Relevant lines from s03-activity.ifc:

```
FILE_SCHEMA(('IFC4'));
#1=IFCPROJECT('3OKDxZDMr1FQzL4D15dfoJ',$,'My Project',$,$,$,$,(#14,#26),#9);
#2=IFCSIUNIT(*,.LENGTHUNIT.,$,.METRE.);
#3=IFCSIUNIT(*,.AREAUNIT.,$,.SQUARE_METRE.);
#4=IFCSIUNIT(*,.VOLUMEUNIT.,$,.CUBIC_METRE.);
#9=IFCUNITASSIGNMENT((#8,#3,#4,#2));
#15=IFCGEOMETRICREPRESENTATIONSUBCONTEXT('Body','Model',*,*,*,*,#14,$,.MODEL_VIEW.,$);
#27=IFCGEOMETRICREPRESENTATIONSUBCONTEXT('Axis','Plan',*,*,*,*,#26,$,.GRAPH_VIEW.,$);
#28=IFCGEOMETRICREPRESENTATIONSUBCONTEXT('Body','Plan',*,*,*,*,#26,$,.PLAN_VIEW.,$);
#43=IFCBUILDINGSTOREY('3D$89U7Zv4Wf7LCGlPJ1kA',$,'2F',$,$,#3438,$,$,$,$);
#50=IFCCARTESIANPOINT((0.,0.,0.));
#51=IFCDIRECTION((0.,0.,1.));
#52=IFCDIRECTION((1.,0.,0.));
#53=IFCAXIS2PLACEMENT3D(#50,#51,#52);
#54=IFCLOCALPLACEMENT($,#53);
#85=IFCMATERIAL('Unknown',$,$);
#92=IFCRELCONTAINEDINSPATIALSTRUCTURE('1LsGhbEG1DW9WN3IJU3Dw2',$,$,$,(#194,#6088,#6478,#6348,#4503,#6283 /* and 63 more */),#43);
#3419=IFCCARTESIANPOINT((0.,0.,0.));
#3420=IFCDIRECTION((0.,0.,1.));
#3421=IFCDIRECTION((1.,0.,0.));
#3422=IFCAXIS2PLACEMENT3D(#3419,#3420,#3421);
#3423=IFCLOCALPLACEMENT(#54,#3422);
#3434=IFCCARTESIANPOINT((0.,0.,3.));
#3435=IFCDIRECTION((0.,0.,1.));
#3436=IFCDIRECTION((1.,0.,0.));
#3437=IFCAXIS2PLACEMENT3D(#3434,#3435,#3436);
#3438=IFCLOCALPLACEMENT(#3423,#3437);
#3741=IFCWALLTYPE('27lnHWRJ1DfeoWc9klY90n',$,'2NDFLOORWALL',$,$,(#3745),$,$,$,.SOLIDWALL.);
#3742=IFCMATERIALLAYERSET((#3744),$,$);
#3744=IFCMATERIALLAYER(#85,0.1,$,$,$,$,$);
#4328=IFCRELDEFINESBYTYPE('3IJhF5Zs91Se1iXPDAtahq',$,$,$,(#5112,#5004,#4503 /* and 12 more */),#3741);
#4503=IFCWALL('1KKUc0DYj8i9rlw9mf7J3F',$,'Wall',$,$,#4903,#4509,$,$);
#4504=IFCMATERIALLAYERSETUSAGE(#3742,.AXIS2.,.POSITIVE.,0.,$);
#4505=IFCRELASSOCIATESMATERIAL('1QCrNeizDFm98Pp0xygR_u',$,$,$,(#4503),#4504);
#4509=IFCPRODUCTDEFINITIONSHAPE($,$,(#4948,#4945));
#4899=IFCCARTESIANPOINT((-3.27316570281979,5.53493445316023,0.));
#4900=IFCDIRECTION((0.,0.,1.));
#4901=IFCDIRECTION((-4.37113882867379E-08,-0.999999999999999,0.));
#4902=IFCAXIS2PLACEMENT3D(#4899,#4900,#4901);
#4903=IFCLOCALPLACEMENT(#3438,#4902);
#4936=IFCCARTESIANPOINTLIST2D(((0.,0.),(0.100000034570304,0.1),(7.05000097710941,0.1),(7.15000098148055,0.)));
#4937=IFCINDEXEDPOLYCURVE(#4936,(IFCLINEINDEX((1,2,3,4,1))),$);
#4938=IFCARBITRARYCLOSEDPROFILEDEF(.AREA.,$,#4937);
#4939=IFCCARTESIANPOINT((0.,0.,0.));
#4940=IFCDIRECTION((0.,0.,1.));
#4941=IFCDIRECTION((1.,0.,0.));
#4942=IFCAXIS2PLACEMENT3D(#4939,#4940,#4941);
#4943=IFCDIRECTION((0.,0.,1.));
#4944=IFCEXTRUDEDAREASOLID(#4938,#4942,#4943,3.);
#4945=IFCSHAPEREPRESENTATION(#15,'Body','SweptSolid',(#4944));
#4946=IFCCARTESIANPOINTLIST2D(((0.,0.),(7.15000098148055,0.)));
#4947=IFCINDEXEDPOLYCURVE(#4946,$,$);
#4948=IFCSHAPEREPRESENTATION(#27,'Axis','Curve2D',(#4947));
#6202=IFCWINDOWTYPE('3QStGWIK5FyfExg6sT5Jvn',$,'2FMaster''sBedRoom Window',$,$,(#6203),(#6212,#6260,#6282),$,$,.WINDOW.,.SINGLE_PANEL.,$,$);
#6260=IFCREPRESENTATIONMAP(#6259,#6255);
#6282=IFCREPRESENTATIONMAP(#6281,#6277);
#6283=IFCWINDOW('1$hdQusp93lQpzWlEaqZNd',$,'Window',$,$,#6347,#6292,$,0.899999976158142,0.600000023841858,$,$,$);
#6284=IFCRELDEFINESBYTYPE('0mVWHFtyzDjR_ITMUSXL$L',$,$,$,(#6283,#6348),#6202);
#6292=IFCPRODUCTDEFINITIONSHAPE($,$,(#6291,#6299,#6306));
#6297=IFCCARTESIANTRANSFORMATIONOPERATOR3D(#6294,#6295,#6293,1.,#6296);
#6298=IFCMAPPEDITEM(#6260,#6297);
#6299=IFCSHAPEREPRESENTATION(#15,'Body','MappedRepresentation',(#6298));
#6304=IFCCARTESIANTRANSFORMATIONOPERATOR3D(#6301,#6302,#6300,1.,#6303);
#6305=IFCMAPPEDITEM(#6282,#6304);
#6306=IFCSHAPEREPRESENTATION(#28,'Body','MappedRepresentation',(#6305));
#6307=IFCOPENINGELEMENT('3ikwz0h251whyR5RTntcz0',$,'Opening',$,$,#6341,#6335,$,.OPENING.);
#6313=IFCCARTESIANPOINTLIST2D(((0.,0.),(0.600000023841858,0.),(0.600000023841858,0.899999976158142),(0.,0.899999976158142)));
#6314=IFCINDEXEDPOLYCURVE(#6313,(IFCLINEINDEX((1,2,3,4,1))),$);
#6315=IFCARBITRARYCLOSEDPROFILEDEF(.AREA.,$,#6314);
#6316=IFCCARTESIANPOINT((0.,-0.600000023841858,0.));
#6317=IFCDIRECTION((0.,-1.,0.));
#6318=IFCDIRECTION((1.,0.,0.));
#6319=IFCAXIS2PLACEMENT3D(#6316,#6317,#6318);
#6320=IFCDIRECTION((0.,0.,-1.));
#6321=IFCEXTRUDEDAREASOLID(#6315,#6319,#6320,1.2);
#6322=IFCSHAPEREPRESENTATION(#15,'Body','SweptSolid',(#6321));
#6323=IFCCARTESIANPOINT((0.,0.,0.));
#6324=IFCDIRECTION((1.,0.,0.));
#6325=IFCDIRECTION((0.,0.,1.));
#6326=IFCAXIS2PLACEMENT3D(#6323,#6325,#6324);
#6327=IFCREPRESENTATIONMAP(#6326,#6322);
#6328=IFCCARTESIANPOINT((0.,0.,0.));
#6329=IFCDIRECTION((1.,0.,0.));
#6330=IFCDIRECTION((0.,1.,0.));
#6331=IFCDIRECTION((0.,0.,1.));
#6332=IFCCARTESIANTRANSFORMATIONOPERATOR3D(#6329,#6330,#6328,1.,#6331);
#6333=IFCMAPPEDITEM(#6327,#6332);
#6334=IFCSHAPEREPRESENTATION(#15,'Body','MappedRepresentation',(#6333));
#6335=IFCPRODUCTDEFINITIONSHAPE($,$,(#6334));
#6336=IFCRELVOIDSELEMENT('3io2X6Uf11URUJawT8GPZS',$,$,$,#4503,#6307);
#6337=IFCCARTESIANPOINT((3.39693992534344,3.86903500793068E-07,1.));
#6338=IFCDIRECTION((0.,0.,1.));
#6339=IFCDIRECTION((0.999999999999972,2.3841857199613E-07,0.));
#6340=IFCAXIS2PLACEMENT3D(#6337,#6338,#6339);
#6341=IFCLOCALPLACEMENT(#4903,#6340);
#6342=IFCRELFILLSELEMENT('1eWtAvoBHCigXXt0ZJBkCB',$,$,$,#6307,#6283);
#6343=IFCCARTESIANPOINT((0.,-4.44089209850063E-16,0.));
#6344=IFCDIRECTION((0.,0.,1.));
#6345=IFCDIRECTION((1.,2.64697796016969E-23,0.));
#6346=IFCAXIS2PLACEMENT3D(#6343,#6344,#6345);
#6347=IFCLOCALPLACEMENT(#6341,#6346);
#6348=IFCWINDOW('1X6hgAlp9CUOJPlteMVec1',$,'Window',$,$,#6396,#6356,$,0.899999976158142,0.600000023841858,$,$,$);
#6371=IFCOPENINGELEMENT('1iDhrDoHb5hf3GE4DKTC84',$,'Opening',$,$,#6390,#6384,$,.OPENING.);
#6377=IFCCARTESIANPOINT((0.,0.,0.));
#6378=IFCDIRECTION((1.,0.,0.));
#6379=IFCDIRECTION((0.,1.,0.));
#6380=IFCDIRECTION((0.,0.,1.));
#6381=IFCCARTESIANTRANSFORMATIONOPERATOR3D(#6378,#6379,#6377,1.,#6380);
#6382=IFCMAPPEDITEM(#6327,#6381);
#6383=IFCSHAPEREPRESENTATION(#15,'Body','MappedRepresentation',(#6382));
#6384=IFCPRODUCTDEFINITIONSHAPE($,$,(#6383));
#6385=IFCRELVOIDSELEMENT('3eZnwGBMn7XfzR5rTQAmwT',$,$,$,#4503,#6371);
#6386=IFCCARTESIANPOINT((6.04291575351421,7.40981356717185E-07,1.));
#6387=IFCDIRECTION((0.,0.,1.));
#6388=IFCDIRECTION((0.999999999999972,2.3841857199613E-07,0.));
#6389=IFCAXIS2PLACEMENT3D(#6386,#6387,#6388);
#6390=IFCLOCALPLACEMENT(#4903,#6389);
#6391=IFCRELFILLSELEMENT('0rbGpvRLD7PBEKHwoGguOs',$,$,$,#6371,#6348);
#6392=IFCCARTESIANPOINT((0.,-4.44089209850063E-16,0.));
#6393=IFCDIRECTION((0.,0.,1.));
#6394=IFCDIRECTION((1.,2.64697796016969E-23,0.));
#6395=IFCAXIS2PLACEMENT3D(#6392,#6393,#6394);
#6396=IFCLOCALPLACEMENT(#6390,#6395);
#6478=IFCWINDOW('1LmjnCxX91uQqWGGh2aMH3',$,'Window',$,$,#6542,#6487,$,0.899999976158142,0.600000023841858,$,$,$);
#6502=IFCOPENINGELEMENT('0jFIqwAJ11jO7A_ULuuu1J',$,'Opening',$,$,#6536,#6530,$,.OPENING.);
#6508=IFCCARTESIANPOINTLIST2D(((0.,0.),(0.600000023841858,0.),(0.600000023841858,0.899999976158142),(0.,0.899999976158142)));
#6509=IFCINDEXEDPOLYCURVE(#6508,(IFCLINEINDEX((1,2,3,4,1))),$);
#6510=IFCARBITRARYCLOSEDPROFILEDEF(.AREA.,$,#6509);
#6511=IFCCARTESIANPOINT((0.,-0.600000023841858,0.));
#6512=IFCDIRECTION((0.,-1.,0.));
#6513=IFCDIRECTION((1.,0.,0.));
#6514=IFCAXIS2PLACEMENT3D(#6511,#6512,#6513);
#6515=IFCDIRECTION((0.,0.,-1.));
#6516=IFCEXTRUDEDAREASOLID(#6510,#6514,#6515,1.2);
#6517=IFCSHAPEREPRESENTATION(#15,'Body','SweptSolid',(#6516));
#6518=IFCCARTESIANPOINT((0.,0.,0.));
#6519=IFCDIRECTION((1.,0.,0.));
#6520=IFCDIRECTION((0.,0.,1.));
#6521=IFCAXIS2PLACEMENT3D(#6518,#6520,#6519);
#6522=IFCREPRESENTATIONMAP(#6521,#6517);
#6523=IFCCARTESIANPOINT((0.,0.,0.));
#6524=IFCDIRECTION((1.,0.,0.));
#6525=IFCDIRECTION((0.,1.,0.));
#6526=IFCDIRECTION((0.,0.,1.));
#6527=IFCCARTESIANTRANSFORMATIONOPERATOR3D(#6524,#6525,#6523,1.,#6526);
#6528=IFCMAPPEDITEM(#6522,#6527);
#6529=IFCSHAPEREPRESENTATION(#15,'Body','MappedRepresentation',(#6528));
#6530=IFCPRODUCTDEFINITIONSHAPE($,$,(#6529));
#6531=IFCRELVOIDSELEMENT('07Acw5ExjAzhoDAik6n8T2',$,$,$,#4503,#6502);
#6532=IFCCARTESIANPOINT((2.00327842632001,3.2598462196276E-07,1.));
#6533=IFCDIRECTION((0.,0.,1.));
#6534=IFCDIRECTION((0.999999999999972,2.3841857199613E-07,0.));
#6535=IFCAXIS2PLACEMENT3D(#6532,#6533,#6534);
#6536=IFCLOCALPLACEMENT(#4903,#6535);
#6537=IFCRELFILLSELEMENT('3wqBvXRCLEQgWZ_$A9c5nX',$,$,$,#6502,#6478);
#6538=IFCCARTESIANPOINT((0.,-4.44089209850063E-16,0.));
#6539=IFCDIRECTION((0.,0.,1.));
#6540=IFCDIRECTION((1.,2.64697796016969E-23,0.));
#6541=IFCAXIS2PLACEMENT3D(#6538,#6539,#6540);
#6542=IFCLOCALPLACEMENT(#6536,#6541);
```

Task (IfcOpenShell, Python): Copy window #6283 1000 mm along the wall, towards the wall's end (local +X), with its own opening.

```python
import ifcopenshell
import ifcopenshell.api.feature
import ifcopenshell.api.geometry
import ifcopenshell.api.root
import ifcopenshell.geom
import ifcopenshell.util.element
import ifcopenshell.util.placement
import ifcopenshell.util.shape
import ifcopenshell.util.unit

model = ifcopenshell.open("s03-activity.ifc")
unit_scale = ifcopenshell.util.unit.calculate_unit_scale(model)
settings = ifcopenshell.geom.settings()


def volume(element):
    """Net volume in cubic metres, openings subtracted."""
    shape = ifcopenshell.geom.create_shape(settings, element)
    return ifcopenshell.util.shape.get_volume(shape.geometry)


window = model.by_id(6283)
opening = window.FillsVoids[0].RelatingOpeningElement
wall = opening.VoidsElements[0].RelatingBuildingElement
before = volume(wall)
shift = ifcopenshell.util.placement.get_local_placement(wall.ObjectPlacement)[:3, 0] * 1 / unit_scale

# copy_class copies the void relationship, type, container and properties, but no geometry.
new_opening = ifcopenshell.api.root.copy_class(model, product=opening)
new_opening.Representation = ifcopenshell.util.element.copy_deep(
    model, opening.Representation, exclude=["IfcGeometricRepresentationContext", "IfcRepresentationMap"]
)
new_window = ifcopenshell.api.root.copy_class(model, product=window)
new_window.Representation = ifcopenshell.util.element.copy_deep(
    model, window.Representation, exclude=["IfcGeometricRepresentationContext", "IfcRepresentationMap"]
)
ifcopenshell.api.feature.add_filling(model, opening=new_opening, element=new_window)

for old, new in ((opening, new_opening), (window, new_window)):
    matrix = ifcopenshell.util.placement.get_local_placement(old.ObjectPlacement)
    matrix[:3, 3] += shift
    ifcopenshell.api.geometry.edit_object_placement(model, product=new, matrix=matrix, is_si=False)

after = volume(wall)

print(f"wall volume {before:.3f} -> {after:.3f} m3")

model.write("s03-activity_edited.ifc")
```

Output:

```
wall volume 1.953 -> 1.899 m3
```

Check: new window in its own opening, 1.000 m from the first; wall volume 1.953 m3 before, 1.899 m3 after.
